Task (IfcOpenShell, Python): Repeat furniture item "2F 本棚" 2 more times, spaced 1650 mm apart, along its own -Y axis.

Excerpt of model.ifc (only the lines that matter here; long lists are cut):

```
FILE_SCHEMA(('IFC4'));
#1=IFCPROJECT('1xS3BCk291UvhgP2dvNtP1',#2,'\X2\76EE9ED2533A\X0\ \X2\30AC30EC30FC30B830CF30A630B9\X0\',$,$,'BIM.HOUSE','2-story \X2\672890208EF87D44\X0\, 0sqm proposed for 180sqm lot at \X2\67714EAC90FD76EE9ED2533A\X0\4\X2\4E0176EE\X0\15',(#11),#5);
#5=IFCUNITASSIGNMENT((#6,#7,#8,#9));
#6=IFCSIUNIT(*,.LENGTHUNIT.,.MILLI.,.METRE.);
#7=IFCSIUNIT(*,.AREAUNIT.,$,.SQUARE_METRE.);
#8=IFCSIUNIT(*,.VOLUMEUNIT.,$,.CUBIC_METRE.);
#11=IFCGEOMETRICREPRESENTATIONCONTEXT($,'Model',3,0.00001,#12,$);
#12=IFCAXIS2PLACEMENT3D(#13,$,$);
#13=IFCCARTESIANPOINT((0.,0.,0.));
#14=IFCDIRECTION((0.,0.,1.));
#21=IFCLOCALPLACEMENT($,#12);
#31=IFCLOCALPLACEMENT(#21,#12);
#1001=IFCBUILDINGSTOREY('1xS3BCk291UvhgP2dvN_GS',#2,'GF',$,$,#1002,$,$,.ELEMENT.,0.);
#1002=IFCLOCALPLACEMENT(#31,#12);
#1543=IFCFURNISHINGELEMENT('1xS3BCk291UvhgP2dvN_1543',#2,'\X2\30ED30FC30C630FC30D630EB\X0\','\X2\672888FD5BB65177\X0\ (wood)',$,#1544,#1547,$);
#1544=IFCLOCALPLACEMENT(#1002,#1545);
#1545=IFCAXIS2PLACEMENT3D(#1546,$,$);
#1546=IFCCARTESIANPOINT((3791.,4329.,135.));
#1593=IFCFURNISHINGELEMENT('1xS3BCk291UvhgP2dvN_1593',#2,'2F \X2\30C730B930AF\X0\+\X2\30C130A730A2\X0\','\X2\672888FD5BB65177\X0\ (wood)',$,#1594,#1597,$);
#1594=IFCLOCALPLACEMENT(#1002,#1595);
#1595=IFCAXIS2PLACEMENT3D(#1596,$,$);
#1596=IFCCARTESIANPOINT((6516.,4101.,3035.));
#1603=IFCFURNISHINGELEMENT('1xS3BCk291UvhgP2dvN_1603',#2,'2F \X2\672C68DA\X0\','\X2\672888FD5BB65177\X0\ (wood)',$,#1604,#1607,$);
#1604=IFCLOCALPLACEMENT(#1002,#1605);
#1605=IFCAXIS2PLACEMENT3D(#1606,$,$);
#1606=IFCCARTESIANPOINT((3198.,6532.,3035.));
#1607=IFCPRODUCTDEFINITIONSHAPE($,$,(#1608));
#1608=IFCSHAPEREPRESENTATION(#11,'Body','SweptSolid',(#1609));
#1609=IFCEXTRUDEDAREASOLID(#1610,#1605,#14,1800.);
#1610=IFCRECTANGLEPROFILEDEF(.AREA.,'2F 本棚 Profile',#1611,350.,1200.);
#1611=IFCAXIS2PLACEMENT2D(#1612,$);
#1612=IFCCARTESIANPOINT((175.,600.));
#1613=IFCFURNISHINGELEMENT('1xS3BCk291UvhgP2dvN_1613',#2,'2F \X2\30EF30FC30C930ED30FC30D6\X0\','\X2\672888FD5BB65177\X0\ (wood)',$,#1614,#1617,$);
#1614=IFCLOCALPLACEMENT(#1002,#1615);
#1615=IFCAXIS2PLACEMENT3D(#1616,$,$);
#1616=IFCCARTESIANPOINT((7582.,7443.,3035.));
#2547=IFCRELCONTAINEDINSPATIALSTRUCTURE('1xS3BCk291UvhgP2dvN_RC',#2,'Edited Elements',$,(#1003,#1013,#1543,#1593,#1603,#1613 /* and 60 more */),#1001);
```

```python
import ifcopenshell
import ifcopenshell.api.geometry
import ifcopenshell.api.root
import ifcopenshell.util.element
import ifcopenshell.util.placement

model = ifcopenshell.open("model.ifc")


def reuse_history(source, copy):
    """copy_class also copies each property set's owner history, people and application; keep the originals."""
    for rel in copy.IsDefinedBy:
        if rel.is_a("IfcRelDefinesByProperties") and (history := rel.RelatingPropertyDefinition.OwnerHistory):
            rel.RelatingPropertyDefinition.OwnerHistory = source.OwnerHistory
            ifcopenshell.util.element.remove_deep2(model, history)


source = model.by_guid("1xS3BCk291UvhgP2dvN_1603")
base = ifcopenshell.util.placement.get_local_placement(source.ObjectPlacement)
step = -base[:3, 1] * 1650.0

for i in range(1, 3):
    copy = ifcopenshell.api.root.copy_class(model, product=source)
    copy.Representation = ifcopenshell.util.element.copy_deep(
        model, source.Representation, exclude=["IfcGeometricRepresentationContext", "IfcRepresentationMap"]
    )
    reuse_history(source, copy)
    matrix = base.copy()
    matrix[:3, 3] += i * step
    print("added at", matrix[:3, 3].round(3) + 0.0)
    ifcopenshell.api.geometry.edit_object_placement(model, product=copy, matrix=matrix, is_si=False)

model.write("model_updated.ifc")
```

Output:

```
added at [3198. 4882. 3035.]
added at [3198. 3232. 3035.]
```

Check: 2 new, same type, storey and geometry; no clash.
